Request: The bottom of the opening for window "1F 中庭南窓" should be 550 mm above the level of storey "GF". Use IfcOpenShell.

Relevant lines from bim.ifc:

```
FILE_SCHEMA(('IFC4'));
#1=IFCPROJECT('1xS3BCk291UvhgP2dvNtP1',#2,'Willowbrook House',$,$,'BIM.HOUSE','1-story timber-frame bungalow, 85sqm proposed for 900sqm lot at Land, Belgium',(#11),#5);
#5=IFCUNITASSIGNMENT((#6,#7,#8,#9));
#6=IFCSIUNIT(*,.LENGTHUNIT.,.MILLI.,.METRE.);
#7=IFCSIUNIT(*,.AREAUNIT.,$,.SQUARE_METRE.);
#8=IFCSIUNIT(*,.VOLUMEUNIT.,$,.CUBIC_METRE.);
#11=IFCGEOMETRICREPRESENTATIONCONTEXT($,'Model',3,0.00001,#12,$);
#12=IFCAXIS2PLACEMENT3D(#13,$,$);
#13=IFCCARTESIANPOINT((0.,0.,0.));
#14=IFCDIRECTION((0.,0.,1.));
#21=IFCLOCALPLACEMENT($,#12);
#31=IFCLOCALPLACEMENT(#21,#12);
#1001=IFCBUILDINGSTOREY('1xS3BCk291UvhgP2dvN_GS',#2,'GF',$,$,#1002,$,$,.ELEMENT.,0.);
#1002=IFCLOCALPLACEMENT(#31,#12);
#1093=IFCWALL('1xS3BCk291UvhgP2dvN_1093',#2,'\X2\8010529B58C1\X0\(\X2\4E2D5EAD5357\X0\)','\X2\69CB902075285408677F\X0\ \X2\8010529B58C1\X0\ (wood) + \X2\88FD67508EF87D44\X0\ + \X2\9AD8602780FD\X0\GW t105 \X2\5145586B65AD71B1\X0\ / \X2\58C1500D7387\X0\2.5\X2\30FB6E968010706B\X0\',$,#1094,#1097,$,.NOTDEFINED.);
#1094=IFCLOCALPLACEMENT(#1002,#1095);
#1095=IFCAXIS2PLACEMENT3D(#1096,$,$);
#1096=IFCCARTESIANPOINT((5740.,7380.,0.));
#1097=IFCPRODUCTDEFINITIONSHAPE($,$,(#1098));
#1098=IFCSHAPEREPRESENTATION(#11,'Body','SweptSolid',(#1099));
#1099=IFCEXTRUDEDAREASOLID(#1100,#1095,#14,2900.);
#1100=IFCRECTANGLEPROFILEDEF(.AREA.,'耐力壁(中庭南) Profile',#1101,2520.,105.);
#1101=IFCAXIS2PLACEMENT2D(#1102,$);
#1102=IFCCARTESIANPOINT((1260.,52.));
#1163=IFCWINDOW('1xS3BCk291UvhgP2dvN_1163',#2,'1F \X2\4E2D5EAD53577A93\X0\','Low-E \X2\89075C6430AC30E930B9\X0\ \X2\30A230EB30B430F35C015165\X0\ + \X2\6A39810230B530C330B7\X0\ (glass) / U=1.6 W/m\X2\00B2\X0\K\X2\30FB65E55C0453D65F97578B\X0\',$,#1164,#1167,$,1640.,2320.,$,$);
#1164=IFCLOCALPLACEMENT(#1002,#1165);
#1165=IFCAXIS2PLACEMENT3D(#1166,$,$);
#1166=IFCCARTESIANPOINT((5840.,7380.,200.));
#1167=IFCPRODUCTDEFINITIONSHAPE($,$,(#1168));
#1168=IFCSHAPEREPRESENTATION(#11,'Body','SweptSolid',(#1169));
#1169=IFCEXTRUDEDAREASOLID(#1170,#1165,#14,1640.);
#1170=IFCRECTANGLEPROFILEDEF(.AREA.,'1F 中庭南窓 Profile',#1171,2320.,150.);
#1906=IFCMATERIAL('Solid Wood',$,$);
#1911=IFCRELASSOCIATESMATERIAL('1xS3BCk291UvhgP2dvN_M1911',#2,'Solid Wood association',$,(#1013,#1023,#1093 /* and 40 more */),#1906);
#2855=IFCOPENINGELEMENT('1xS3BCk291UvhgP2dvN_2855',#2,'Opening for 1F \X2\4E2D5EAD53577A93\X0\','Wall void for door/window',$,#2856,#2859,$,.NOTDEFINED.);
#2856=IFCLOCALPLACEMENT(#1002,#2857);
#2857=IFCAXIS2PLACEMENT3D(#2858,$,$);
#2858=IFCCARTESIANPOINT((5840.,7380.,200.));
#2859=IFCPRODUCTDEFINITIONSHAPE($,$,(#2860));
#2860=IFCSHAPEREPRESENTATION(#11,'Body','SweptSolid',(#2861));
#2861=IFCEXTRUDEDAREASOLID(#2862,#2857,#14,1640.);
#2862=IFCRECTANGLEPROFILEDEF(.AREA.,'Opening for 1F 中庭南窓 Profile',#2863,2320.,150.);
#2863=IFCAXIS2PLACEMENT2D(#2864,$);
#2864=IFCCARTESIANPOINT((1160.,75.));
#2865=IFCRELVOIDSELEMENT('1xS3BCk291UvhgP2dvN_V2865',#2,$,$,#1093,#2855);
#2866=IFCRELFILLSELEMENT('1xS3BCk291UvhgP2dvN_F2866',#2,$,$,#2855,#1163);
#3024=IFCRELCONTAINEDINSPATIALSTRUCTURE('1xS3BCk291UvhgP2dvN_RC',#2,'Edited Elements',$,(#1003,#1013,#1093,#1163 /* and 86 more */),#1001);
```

```python
import numpy as np
import ifcopenshell
import ifcopenshell.api.geometry
import ifcopenshell.geom
import ifcopenshell.util.element
import ifcopenshell.util.placement
import ifcopenshell.util.shape
import ifcopenshell.util.unit

model = ifcopenshell.open("bim.ifc")
unit_scale = ifcopenshell.util.unit.calculate_unit_scale(model)

window = model.by_guid("1xS3BCk291UvhgP2dvN_1163")
opening = window.FillsVoids[0].RelatingOpeningElement
storey = ifcopenshell.util.element.get_container(window, ifc_class="IfcBuildingStorey")
level = ifcopenshell.util.placement.get_local_placement(storey.ObjectPlacement)[2, 3]

# The opening's origin need not be at the sill, so measure its lowest point.
shape = ifcopenshell.geom.create_shape(ifcopenshell.geom.settings(), opening)
bottom = ifcopenshell.util.shape.get_shape_bottom_elevation(shape, shape.geometry) / unit_scale
dz = level + 550.0 - bottom

shift = np.array([0.0, 0.0, dz])
# The window is not placed relative to its opening, so move both.
for product in (opening, window):
    matrix = ifcopenshell.util.placement.get_local_placement(product.ObjectPlacement)
    matrix[:3, 3] += shift
    ifcopenshell.api.geometry.edit_object_placement(model, product=product, matrix=matrix, is_si=False)

print(f"moved by {dz * unit_scale:+.3f} m")

model.write("bim_v2.ifc")
```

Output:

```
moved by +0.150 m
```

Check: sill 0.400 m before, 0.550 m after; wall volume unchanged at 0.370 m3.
